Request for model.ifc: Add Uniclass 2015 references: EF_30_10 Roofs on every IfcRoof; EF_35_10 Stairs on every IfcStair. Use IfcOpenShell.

First a look at what the model holds.

```python
import ifcopenshell

model = ifcopenshell.open("model.ifc")
print(model.schema)
print("classifications:", [c.Name for c in model.by_type("IfcClassification")])
for ifc_class in ("IfcDoor", "IfcRoof", "IfcStair", "IfcWall", "IfcWindow"):
    print(ifc_class, len(model.by_type(ifc_class)))
```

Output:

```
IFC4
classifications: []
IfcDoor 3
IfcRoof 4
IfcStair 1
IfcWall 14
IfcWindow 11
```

```python
import ifcopenshell
import ifcopenshell.api.classification

model = ifcopenshell.open("model.ifc")

system = ifcopenshell.api.classification.add_classification(model, classification="Uniclass 2015")

codes = {
    "IfcRoof": ("EF_30_10", "Roofs"),
    "IfcStair": ("EF_35_10", "Stairs"),
}
for ifc_class, (code, name) in codes.items():
    products = model.by_type(ifc_class)
    ifcopenshell.api.classification.add_reference(
        model, products=products, classification=system, identification=code, name=name
    )
    print(code, len(products))

model.write("model_updated.ifc")
```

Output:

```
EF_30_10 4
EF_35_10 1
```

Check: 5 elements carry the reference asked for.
